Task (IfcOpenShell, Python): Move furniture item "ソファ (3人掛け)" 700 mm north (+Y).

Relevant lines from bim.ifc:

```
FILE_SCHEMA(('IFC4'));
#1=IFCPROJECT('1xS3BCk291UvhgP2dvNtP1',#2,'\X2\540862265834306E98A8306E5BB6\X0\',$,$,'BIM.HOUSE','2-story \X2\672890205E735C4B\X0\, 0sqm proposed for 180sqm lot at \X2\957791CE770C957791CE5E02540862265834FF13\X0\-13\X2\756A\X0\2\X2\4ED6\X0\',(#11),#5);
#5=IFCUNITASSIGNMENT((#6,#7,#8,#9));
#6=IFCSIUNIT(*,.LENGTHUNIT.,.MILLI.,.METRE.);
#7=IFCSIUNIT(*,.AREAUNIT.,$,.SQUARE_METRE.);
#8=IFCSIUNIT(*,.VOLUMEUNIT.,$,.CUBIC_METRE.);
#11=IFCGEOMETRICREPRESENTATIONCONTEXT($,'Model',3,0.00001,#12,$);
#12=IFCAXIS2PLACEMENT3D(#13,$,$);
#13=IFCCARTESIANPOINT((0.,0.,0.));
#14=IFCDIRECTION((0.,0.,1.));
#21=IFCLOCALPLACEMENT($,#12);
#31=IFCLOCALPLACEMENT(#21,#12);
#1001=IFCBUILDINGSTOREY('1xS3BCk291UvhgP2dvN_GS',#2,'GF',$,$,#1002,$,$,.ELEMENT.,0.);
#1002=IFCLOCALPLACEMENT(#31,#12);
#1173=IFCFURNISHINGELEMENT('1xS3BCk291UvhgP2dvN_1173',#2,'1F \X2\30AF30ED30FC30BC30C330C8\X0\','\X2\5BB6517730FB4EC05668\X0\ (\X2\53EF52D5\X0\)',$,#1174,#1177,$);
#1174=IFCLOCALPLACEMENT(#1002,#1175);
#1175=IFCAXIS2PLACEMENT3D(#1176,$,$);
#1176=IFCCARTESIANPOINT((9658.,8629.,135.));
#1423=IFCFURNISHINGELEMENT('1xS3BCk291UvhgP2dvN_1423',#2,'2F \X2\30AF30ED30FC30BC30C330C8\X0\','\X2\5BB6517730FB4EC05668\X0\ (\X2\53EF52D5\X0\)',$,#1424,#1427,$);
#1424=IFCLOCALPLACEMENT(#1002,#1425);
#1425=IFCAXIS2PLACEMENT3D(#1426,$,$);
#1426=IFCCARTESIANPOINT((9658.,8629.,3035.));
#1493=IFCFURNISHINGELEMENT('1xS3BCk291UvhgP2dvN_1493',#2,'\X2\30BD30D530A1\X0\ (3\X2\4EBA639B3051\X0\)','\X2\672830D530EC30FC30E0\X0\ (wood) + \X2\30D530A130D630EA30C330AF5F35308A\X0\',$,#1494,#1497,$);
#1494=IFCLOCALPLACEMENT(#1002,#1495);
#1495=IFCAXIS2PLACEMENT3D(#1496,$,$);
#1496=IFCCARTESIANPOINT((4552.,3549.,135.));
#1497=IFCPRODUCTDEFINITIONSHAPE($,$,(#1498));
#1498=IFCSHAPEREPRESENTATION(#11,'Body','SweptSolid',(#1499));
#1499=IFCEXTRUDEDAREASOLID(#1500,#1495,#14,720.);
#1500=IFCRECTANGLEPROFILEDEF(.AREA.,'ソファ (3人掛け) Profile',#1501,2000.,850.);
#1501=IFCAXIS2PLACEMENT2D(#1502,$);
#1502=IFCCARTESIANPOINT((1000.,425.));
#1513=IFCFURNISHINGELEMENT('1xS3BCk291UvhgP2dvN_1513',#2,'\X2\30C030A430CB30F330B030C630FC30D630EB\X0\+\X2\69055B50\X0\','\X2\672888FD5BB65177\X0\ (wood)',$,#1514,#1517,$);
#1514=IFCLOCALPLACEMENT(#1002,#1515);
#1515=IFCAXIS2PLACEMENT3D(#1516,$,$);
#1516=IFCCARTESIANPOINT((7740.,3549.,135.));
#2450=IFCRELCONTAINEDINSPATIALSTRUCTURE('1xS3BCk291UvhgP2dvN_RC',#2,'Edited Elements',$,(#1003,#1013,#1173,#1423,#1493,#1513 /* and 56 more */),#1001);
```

```python
import ifcopenshell
import ifcopenshell.api.geometry
import ifcopenshell.util.placement
import ifcopenshell.util.unit

model = ifcopenshell.open("bim.ifc")
unit_scale = ifcopenshell.util.unit.calculate_unit_scale(model)

item = model.by_guid("1xS3BCk291UvhgP2dvN_1493")
matrix = ifcopenshell.util.placement.get_local_placement(item.ObjectPlacement)
matrix[1, 3] += 0.7 / unit_scale
ifcopenshell.api.geometry.edit_object_placement(model, product=item, matrix=matrix, is_si=False)

print(ifcopenshell.util.placement.get_local_placement(item.ObjectPlacement).round(3) + 0.0)

model.write("bim_edited.ifc")
```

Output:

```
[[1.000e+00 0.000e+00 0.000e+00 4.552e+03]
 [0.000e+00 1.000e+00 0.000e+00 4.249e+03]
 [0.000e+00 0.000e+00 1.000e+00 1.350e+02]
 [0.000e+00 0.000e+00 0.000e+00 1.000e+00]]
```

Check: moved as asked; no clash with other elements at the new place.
